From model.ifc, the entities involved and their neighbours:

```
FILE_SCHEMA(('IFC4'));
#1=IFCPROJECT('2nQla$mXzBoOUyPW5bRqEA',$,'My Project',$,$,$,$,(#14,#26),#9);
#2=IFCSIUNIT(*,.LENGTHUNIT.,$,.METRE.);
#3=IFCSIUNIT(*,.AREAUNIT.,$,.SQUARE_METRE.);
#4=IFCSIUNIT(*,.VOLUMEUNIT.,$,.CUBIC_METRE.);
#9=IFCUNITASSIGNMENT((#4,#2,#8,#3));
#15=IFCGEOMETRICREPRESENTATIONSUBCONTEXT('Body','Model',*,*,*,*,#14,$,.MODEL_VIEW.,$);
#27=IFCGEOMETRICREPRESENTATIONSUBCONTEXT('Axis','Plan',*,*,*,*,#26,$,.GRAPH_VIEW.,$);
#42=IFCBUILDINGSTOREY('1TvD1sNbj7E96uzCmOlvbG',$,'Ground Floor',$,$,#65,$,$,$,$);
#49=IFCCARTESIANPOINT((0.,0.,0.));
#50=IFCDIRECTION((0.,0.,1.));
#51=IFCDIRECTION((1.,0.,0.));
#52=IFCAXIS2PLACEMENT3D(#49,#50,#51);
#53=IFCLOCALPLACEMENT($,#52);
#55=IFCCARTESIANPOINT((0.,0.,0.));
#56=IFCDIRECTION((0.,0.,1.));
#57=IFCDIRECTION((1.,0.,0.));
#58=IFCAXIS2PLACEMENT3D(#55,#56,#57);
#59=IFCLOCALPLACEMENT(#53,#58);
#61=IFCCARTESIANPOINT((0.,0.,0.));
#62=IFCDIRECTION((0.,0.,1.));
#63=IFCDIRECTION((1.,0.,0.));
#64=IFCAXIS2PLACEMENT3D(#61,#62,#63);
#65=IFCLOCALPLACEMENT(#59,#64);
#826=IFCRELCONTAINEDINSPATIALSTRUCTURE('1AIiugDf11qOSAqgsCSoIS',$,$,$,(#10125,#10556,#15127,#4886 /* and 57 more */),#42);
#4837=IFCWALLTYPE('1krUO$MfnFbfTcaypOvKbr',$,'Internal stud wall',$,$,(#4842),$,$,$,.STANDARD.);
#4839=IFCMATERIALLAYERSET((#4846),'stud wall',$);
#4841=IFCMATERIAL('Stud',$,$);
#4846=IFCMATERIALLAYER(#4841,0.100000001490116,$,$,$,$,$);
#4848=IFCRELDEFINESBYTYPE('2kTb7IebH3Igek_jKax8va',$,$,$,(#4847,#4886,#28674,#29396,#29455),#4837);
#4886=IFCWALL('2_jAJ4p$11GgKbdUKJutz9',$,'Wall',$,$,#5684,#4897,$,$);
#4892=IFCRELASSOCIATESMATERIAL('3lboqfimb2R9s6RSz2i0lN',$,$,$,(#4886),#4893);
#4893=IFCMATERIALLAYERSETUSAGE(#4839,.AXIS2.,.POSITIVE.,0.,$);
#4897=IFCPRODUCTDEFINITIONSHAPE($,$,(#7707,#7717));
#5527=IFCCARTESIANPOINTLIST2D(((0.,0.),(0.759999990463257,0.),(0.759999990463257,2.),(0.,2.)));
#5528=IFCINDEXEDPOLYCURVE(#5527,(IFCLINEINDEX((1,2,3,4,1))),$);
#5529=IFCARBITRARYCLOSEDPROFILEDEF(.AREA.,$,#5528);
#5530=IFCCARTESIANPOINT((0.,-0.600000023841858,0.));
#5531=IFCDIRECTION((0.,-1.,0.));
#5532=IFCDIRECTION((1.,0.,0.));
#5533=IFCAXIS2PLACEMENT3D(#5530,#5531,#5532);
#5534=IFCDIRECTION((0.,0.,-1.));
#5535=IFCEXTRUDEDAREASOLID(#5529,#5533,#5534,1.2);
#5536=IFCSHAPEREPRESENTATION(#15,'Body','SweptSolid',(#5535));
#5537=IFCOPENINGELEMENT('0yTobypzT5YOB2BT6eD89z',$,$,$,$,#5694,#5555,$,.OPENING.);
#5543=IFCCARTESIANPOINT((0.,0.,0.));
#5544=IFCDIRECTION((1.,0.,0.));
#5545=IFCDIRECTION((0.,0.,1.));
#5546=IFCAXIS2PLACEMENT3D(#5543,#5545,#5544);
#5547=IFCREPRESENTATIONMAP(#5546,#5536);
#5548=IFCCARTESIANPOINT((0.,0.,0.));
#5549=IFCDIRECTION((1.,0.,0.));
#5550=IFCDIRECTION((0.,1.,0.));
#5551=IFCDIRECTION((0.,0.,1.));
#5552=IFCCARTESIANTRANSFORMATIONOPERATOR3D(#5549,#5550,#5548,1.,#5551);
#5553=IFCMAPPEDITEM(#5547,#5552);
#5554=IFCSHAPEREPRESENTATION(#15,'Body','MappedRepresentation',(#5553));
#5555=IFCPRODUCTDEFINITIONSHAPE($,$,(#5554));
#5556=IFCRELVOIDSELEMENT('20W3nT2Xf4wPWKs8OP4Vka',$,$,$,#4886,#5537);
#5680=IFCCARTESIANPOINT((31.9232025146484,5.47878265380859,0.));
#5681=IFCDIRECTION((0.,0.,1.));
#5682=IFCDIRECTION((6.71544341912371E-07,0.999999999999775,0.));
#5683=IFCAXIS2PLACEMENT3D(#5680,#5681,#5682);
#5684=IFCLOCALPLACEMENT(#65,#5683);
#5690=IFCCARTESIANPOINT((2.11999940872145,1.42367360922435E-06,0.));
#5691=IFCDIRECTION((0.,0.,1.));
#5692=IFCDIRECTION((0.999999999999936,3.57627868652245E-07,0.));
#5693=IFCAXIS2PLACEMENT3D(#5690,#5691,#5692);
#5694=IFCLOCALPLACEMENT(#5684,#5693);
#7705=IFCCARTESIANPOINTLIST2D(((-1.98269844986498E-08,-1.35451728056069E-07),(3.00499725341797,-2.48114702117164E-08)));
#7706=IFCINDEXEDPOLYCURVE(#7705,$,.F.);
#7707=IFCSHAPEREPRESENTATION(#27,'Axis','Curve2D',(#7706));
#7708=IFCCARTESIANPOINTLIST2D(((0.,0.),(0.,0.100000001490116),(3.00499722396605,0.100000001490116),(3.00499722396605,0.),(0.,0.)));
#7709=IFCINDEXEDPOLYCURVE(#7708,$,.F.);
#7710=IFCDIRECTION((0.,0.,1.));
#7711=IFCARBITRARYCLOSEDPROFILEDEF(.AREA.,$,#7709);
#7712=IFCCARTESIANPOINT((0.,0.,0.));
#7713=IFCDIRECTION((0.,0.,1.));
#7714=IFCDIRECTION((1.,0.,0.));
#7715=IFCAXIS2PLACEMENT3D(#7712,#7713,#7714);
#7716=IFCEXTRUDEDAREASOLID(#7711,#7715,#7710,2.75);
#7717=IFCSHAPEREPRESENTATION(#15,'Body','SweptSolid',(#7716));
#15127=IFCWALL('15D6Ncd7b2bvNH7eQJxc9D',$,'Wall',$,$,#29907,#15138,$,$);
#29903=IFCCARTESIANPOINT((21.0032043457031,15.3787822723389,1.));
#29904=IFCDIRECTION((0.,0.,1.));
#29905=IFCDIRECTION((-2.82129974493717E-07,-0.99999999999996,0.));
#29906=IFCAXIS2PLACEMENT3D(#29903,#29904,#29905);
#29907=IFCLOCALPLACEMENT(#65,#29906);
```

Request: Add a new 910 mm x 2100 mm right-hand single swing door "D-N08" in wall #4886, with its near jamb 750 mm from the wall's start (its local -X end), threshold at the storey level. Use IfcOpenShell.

```python
import numpy as np
import ifcopenshell
import ifcopenshell.api.feature
import ifcopenshell.api.geometry
import ifcopenshell.api.root
import ifcopenshell.api.spatial
import ifcopenshell.geom
import ifcopenshell.util.element
import ifcopenshell.util.placement
import ifcopenshell.util.representation
import ifcopenshell.util.shape
import ifcopenshell.util.unit

model = ifcopenshell.open("model.ifc")
unit_scale = ifcopenshell.util.unit.calculate_unit_scale(model)
settings = ifcopenshell.geom.settings()


def volume(element):
    """Net volume in cubic metres, openings subtracted."""
    shape = ifcopenshell.geom.create_shape(settings, element)
    return ifcopenshell.util.shape.get_volume(shape.geometry)


wall = model.by_guid("2_jAJ4p$11GgKbdUKJutz9")
storey = ifcopenshell.util.element.get_container(wall, ifc_class="IfcBuildingStorey")
context = ifcopenshell.util.representation.get_context(model, "Model", "Body", "MODEL_VIEW")
before = volume(wall)

width, height, from_end, sill = 0.91, 2.1, 0.75, 0.0  # metres

# The wall runs along its own X axis, and the end named is its -X end.
wall_shape = ifcopenshell.geom.create_shape(settings, wall)
x, y, z = ifcopenshell.util.shape.get_vertices(wall_shape.geometry).T
start = x.min() + from_end
face, thickness = float(y.min()), float(y.max() - y.min())
wall_matrix = ifcopenshell.util.placement.get_local_placement(wall.ObjectPlacement)
level = ifcopenshell.util.placement.get_local_placement(storey.ObjectPlacement)[2, 3]


def in_wall(x, y):
    """Placement at x, y metres in the wall's axes, at sill height."""
    matrix = wall_matrix.copy()
    matrix[:, 3] = wall_matrix @ np.array([x / unit_scale, y / unit_scale, 0.0, 1.0])
    matrix[2, 3] = level + sill / unit_scale
    return matrix


# Opening: a box that overshoots both wall faces by 50 mm.
opening = ifcopenshell.api.root.create_entity(model, ifc_class="IfcOpeningElement", predefined_type="OPENING")
box = ifcopenshell.api.geometry.add_wall_representation(
    model, context=context, length=width, height=height, thickness=thickness + 0.1
)
ifcopenshell.api.geometry.assign_representation(model, product=opening, representation=box)
ifcopenshell.api.geometry.edit_object_placement(model, product=opening, matrix=in_wall(start, face - 0.05), is_si=False)
ifcopenshell.api.feature.add_feature(model, feature=opening, element=wall)

door = ifcopenshell.api.root.create_entity(model, ifc_class="IfcDoor", name="D-N08", predefined_type="DOOR")
door.OverallWidth, door.OverallHeight = width / unit_scale, height / unit_scale
door.OperationType = "SINGLE_SWING_RIGHT"
body = ifcopenshell.api.geometry.add_door_representation(
    model,
    context=context,
    overall_width=door.OverallWidth,
    overall_height=door.OverallHeight,
    operation_type="SINGLE_SWING_RIGHT",
    lining_properties={"LiningDepth": thickness / unit_scale, "ThresholdDepth": thickness / unit_scale},
)
ifcopenshell.api.geometry.assign_representation(model, product=door, representation=body)
ifcopenshell.api.spatial.assign_container(model, products=[door], relating_structure=storey)
ifcopenshell.api.feature.add_filling(model, opening=opening, element=door)

# The lining spans the wall, so the door starts at the wall face.
ifcopenshell.api.geometry.edit_object_placement(model, product=door, matrix=in_wall(start, face), is_si=False)

after = volume(wall)

print(f"wall volume {before:.3f} -> {after:.3f} m3")

model.write("model_rev.ifc")
```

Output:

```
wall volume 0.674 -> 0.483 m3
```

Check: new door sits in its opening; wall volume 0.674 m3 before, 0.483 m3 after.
